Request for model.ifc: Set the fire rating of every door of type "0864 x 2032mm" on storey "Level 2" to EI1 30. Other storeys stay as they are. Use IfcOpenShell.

First a look at what the model holds.

```python
import ifcopenshell
import ifcopenshell.util.element

model = ifcopenshell.open("model.ifc")
print(model.schema)
storey = next(s for s in model.by_type("IfcBuildingStorey") if s.Name == "Level 2")
doors = [e for e in ifcopenshell.util.element.get_decomposition(storey) if e.is_a("IfcDoor")]
seen = {}
for e in doors:
    element_type = ifcopenshell.util.element.get_type(e)
    key = (element_type.Name if element_type != e and element_type else None, ifcopenshell.util.element.get_pset(e, "Pset_DoorCommon", "FireRating"))
    seen[key] = seen.get(key, 0) + 1
for (name, value), count in sorted(seen.items(), key=str):
    print(count, "x", name, "|", value)
```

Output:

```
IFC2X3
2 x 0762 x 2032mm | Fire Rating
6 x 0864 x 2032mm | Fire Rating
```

```python
import ifcopenshell
import ifcopenshell.api.pset
import ifcopenshell.util.element

model = ifcopenshell.open("model.ifc")

storey = next(s for s in model.by_type("IfcBuildingStorey") if s.Name == "Level 2")
doors = [e for e in ifcopenshell.util.element.get_decomposition(storey) if e.is_a("IfcDoor")]

count = 0
for e in doors:
    element_type = ifcopenshell.util.element.get_type(e)
    if element_type in (None, e) or element_type.Name != "0864 x 2032mm":
        continue
    # add_pset returns the element's existing set when there is one.
    pset = ifcopenshell.api.pset.add_pset(model, product=e, name="Pset_DoorCommon")
    ifcopenshell.api.pset.edit_pset(model, pset=pset, properties={"FireRating": "EI1 30"})
    count += 1

print(count, "doors updated")

model.write("model_edited.ifc")
```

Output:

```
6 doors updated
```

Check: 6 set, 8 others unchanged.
